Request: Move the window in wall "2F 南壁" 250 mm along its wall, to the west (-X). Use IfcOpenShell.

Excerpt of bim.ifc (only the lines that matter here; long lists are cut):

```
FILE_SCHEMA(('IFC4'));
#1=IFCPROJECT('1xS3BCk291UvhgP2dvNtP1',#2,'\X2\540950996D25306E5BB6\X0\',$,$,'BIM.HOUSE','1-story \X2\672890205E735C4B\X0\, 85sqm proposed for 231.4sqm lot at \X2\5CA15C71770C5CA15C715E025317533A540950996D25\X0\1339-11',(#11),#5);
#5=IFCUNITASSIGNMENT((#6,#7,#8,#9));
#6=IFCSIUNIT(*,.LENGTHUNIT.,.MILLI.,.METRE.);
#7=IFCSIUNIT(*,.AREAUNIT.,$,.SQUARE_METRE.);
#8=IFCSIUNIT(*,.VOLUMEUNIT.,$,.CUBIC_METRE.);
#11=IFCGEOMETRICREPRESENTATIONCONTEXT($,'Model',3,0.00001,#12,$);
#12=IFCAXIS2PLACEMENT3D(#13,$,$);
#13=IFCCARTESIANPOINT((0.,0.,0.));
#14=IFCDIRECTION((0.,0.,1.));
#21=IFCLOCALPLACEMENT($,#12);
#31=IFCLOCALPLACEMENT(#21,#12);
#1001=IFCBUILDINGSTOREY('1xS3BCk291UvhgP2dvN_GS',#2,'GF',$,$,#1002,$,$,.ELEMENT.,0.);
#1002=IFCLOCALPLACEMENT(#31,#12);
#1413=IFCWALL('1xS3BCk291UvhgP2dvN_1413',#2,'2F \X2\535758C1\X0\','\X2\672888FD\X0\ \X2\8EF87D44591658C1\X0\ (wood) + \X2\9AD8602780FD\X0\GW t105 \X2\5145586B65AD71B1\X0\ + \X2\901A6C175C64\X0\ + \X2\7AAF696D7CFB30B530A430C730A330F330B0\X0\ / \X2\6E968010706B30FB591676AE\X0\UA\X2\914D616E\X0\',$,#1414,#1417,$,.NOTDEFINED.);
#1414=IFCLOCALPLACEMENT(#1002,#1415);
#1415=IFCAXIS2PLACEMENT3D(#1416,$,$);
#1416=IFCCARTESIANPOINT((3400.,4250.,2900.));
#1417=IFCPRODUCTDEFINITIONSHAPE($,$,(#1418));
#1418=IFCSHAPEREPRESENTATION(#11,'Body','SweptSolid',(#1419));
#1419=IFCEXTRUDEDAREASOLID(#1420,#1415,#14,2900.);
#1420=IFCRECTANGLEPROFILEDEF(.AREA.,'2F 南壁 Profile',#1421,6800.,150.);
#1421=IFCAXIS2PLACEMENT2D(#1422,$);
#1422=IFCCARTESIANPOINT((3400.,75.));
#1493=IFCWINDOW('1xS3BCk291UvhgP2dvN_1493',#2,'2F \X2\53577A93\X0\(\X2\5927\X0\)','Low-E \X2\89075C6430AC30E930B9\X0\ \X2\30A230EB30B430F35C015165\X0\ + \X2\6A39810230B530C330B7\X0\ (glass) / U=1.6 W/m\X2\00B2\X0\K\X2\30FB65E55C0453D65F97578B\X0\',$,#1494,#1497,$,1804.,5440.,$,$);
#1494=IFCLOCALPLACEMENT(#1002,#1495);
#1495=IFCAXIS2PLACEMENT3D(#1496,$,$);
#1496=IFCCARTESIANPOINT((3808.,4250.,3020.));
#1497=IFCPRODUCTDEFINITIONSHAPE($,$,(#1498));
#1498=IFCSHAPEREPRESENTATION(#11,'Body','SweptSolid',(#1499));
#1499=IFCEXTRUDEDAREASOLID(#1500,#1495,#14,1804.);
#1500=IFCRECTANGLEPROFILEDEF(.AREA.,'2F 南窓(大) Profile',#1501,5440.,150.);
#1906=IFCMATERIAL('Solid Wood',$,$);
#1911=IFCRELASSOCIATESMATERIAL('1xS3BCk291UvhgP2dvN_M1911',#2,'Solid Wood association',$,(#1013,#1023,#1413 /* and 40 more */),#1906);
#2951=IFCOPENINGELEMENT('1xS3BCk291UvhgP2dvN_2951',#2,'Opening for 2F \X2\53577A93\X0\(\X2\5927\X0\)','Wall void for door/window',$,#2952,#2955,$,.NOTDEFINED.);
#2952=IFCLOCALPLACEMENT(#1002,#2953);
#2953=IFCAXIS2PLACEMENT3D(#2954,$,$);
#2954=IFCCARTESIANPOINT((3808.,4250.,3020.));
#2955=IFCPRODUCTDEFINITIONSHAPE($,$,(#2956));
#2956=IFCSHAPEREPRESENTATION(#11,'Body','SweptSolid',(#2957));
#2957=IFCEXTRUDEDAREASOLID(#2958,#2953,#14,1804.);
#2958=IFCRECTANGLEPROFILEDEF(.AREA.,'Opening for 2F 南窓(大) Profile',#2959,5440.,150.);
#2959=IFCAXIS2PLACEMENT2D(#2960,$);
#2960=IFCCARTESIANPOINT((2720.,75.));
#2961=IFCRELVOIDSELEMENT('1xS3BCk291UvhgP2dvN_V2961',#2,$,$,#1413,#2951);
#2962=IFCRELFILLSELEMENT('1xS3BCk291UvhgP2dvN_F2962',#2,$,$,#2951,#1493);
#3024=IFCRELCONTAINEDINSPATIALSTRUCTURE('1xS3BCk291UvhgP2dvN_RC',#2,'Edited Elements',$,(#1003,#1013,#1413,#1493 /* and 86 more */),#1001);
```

```python
import ifcopenshell
import ifcopenshell.api.geometry
import ifcopenshell.util.placement

model = ifcopenshell.open("bim.ifc")

window = model.by_id(1493)
opening = window.FillsVoids[0].RelatingOpeningElement
wall = opening.VoidsElements[0].RelatingBuildingElement

wall_matrix = ifcopenshell.util.placement.get_local_placement(wall.ObjectPlacement)
shift = wall_matrix[:3, 0] * -250.0
before = ifcopenshell.util.placement.get_local_placement(window.ObjectPlacement)[:3, 3].copy()

# The window is not placed relative to its opening, so move both.
for product in (opening, window):
    matrix = ifcopenshell.util.placement.get_local_placement(product.ObjectPlacement)
    matrix[:3, 3] += shift
    ifcopenshell.api.geometry.edit_object_placement(model, product=product, matrix=matrix, is_si=False)

after = ifcopenshell.util.placement.get_local_placement(window.ObjectPlacement)[:3, 3]
print("window moved by", (after - before).round(3) + 0.0)

model.write("bim_rev.ifc")
```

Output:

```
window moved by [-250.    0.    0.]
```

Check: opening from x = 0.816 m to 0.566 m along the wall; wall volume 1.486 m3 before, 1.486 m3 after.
